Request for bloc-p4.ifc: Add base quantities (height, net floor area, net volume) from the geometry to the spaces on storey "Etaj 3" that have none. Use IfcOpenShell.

First a look at what the model holds.

```python
import ifcopenshell
import ifcopenshell.util.element
import ifcopenshell.util.unit

model = ifcopenshell.open("bloc-p4.ifc")
print(model.schema)
for unit_type in ("LENGTHUNIT", "AREAUNIT", "VOLUMEUNIT"):
    print(unit_type, ifcopenshell.util.unit.calculate_unit_scale(model, unit_type))
storey = next(s for s in model.by_type("IfcBuildingStorey") if s.Name == "Etaj 3")
spaces = [e for e in ifcopenshell.util.element.get_decomposition(storey) if e.is_a("IfcSpace")]
for e in sorted(spaces, key=lambda e: e.id()):
    print(e.id(), e.is_a(), e.Name, list(ifcopenshell.util.element.get_psets(e, qtos_only=True)), sep=" | ")
```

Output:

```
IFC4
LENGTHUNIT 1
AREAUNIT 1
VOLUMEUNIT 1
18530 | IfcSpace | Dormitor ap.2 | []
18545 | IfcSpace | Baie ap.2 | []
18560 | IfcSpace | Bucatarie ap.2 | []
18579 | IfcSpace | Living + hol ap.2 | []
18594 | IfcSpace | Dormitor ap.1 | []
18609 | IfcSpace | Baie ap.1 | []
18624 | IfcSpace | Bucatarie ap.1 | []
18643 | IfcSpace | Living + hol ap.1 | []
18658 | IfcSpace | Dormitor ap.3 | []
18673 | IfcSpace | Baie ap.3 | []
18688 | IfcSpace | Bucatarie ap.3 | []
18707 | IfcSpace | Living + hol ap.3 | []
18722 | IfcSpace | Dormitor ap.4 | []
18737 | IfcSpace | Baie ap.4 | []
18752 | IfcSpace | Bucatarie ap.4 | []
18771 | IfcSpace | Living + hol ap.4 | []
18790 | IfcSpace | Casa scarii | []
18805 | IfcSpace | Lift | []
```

```python
import ifcopenshell
import ifcopenshell.api.pset
import ifcopenshell.geom
import ifcopenshell.util.element
import ifcopenshell.util.shape
import ifcopenshell.util.unit

model = ifcopenshell.open("bloc-p4.ifc")
unit_scale = ifcopenshell.util.unit.calculate_unit_scale(model)
area_scale = ifcopenshell.util.unit.calculate_unit_scale(model, "AREAUNIT")
volume_scale = ifcopenshell.util.unit.calculate_unit_scale(model, "VOLUMEUNIT")
settings = ifcopenshell.geom.settings()

storey = next(s for s in model.by_type("IfcBuildingStorey") if s.Name == "Etaj 3")
spaces = [e for e in ifcopenshell.util.element.get_decomposition(storey) if e.is_a("IfcSpace")]

for e in sorted(spaces, key=lambda e: e.id()):
    if ifcopenshell.util.element.get_psets(e, qtos_only=True, should_inherit=False):
        continue
    # Geometry comes back in metres, in the element's own axes.
    shape = ifcopenshell.geom.create_shape(settings, e)
    values = {
        "Height": ifcopenshell.util.shape.get_z(shape.geometry) / unit_scale,
        "NetFloorArea": ifcopenshell.util.shape.get_footprint_area(shape.geometry) / area_scale,
        "NetVolume": ifcopenshell.util.shape.get_volume(shape.geometry) / volume_scale,
    }
    qto = ifcopenshell.api.pset.add_qto(model, product=e, name="Qto_SpaceBaseQuantities")
    ifcopenshell.api.pset.edit_qto(model, qto=qto, properties=values)
    print(e.id(), {k: round(v, 3) for k, v in values.items()})

model.write("bloc-p4_v2.ifc")
```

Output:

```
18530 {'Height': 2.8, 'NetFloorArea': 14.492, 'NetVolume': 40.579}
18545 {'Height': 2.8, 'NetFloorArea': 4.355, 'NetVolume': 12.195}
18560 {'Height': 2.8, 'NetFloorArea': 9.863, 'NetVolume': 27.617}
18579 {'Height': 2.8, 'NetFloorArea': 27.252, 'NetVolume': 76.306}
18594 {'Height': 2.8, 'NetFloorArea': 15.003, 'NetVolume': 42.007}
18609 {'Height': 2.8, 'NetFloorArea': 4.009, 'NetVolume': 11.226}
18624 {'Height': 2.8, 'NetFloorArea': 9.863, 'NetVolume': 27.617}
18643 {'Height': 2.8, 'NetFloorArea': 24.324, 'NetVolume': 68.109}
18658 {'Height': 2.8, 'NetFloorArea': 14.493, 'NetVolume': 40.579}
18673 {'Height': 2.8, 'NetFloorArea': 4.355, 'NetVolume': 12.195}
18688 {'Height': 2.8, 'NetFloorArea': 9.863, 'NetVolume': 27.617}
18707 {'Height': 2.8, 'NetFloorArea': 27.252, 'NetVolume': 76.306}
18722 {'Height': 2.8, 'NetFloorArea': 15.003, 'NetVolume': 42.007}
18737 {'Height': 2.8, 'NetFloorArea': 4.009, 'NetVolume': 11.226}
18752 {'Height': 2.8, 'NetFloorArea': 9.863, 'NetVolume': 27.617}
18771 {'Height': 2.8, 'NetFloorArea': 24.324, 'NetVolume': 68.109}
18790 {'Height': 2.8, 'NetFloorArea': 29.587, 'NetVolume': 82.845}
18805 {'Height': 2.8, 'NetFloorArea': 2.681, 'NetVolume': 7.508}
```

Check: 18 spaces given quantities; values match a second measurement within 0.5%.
